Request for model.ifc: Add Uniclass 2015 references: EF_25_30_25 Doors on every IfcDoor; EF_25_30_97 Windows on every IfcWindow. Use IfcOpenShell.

First a look at what the model holds.

```python
import ifcopenshell

model = ifcopenshell.open("model.ifc")
print(model.schema)
print("classifications:", [c.Name for c in model.by_type("IfcClassification")])
for ifc_class in ("IfcDoor", "IfcRoof", "IfcStair", "IfcWall", "IfcWindow"):
    print(ifc_class, len(model.by_type(ifc_class)))
```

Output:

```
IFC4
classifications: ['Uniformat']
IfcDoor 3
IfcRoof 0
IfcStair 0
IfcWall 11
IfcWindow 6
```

```python
import ifcopenshell
import ifcopenshell.api.classification

model = ifcopenshell.open("model.ifc")

system = ifcopenshell.api.classification.add_classification(model, classification="Uniclass 2015")

codes = {
    "IfcDoor": ("EF_25_30_25", "Doors"),
    "IfcWindow": ("EF_25_30_97", "Windows"),
}
for ifc_class, (code, name) in codes.items():
    products = model.by_type(ifc_class)
    ifcopenshell.api.classification.add_reference(
        model, products=products, classification=system, identification=code, name=name
    )
    print(code, len(products))

model.write("model-out.ifc")
```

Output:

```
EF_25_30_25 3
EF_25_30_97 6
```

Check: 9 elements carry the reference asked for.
